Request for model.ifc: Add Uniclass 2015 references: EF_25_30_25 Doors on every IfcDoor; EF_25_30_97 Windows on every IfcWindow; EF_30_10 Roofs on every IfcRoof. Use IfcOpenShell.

First a look at what the model holds.

```python
import ifcopenshell

model = ifcopenshell.open("model.ifc")
print(model.schema)
print("classifications:", [c.Name for c in model.by_type("IfcClassification")])
for ifc_class in ("IfcDoor", "IfcRoof", "IfcStair", "IfcWall", "IfcWindow"):
    print(ifc_class, len(model.by_type(ifc_class)))
```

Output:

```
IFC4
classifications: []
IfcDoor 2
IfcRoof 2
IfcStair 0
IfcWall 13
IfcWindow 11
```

```python
import ifcopenshell
import ifcopenshell.api.classification

model = ifcopenshell.open("model.ifc")

system = ifcopenshell.api.classification.add_classification(model, classification="Uniclass 2015")

codes = {
    "IfcDoor": ("EF_25_30_25", "Doors"),
    "IfcWindow": ("EF_25_30_97", "Windows"),
    "IfcRoof": ("EF_30_10", "Roofs"),
}
for ifc_class, (code, name) in codes.items():
    products = model.by_type(ifc_class)
    ifcopenshell.api.classification.add_reference(
        model, products=products, classification=system, identification=code, name=name
    )
    print(code, len(products))

model.write("model_rev.ifc")
```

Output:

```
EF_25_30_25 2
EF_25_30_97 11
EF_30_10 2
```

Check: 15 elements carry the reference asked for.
